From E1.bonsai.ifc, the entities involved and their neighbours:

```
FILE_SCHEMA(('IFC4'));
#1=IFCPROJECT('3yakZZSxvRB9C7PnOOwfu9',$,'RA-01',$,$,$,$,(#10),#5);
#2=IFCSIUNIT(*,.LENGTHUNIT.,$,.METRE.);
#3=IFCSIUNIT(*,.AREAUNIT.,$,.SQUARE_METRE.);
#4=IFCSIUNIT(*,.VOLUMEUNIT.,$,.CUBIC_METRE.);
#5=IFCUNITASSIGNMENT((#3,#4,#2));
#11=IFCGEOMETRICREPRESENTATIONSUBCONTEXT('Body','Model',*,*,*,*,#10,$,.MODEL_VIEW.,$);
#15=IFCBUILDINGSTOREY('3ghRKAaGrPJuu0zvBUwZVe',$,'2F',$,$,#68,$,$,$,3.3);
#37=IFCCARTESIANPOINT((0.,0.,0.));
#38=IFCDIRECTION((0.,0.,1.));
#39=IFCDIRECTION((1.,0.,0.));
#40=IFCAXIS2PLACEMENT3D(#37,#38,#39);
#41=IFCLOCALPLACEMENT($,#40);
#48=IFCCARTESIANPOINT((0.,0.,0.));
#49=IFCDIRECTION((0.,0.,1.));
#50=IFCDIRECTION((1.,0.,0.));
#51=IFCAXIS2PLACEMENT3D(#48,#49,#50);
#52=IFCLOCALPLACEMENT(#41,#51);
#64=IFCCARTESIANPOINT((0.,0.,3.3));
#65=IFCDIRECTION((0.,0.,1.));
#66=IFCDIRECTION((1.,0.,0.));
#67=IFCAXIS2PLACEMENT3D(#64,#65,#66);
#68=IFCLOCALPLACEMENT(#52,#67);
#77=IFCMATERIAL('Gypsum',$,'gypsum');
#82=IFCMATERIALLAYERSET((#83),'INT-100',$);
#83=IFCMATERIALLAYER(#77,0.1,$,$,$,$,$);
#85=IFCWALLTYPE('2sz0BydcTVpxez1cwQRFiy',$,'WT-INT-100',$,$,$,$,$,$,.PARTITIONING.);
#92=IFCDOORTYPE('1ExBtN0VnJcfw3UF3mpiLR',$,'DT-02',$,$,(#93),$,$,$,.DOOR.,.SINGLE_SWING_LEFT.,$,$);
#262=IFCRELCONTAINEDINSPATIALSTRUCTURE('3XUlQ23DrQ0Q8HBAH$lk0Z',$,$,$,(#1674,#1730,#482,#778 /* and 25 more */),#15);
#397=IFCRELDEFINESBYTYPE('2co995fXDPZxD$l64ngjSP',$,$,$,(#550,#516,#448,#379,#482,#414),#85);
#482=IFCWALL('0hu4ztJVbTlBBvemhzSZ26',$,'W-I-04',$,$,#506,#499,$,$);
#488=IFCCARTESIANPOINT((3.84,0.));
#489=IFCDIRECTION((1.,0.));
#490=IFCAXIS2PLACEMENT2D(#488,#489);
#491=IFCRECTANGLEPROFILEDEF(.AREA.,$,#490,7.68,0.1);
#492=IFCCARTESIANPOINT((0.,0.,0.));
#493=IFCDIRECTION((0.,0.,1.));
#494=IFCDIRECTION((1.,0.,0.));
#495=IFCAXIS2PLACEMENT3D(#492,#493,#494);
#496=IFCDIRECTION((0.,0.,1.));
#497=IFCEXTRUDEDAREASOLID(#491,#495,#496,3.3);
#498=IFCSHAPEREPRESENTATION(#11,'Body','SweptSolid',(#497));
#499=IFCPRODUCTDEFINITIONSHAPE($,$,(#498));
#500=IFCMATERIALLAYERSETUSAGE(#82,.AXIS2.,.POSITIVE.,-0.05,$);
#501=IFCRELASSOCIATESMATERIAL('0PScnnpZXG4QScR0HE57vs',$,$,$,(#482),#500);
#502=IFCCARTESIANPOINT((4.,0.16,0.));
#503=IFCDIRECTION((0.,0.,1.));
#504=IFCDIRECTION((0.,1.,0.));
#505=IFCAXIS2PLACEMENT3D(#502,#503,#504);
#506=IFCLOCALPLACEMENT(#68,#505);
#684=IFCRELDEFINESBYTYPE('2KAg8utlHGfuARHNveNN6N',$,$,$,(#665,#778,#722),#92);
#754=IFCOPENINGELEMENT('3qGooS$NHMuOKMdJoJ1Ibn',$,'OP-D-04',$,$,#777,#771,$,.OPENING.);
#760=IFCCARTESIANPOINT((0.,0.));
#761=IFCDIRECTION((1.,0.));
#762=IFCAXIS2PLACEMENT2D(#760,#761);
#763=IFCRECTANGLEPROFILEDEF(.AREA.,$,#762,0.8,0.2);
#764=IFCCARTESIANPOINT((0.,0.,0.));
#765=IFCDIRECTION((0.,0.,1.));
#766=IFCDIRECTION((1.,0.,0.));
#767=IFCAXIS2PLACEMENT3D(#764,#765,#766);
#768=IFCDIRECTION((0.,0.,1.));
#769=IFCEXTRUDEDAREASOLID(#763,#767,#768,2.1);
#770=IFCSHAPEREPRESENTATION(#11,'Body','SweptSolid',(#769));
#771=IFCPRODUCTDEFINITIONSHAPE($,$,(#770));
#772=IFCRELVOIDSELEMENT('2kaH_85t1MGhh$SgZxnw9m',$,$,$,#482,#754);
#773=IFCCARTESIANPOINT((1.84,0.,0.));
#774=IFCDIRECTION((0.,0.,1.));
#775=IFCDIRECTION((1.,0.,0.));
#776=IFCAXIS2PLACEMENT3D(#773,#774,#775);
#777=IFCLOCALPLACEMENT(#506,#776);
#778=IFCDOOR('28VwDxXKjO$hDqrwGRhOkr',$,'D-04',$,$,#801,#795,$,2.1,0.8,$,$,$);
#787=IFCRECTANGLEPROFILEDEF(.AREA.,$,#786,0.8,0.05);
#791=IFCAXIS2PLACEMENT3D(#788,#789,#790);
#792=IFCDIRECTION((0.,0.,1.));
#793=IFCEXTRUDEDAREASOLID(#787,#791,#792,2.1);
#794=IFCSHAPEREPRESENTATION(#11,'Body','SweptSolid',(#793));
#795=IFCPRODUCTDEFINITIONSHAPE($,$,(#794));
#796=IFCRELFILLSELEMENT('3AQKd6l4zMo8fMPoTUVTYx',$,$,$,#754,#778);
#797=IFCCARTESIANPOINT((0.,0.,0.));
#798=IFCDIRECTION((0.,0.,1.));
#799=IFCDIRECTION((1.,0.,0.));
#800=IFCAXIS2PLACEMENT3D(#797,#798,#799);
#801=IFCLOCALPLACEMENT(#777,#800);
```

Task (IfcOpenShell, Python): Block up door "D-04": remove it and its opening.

```python
import ifcopenshell
import ifcopenshell.api.feature
import ifcopenshell.api.root
import ifcopenshell.geom
import ifcopenshell.util.shape

model = ifcopenshell.open("E1.bonsai.ifc")
settings = ifcopenshell.geom.settings()


def volume(element):
    """Net volume in cubic metres, openings subtracted."""
    shape = ifcopenshell.geom.create_shape(settings, element)
    return ifcopenshell.util.shape.get_volume(shape.geometry)


door = model.by_guid("28VwDxXKjO$hDqrwGRhOkr")
opening = door.FillsVoids[0].RelatingOpeningElement
wall = opening.VoidsElements[0].RelatingBuildingElement
before = volume(wall)

ifcopenshell.api.root.remove_product(model, product=door)
ifcopenshell.api.feature.remove_feature(model, feature=opening)

after = volume(wall)

print(f"wall volume {before:.3f} -> {after:.3f} m3")

model.write("E1.bonsai-out.ifc")
```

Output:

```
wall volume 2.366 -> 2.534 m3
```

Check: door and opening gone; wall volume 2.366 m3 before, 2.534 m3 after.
